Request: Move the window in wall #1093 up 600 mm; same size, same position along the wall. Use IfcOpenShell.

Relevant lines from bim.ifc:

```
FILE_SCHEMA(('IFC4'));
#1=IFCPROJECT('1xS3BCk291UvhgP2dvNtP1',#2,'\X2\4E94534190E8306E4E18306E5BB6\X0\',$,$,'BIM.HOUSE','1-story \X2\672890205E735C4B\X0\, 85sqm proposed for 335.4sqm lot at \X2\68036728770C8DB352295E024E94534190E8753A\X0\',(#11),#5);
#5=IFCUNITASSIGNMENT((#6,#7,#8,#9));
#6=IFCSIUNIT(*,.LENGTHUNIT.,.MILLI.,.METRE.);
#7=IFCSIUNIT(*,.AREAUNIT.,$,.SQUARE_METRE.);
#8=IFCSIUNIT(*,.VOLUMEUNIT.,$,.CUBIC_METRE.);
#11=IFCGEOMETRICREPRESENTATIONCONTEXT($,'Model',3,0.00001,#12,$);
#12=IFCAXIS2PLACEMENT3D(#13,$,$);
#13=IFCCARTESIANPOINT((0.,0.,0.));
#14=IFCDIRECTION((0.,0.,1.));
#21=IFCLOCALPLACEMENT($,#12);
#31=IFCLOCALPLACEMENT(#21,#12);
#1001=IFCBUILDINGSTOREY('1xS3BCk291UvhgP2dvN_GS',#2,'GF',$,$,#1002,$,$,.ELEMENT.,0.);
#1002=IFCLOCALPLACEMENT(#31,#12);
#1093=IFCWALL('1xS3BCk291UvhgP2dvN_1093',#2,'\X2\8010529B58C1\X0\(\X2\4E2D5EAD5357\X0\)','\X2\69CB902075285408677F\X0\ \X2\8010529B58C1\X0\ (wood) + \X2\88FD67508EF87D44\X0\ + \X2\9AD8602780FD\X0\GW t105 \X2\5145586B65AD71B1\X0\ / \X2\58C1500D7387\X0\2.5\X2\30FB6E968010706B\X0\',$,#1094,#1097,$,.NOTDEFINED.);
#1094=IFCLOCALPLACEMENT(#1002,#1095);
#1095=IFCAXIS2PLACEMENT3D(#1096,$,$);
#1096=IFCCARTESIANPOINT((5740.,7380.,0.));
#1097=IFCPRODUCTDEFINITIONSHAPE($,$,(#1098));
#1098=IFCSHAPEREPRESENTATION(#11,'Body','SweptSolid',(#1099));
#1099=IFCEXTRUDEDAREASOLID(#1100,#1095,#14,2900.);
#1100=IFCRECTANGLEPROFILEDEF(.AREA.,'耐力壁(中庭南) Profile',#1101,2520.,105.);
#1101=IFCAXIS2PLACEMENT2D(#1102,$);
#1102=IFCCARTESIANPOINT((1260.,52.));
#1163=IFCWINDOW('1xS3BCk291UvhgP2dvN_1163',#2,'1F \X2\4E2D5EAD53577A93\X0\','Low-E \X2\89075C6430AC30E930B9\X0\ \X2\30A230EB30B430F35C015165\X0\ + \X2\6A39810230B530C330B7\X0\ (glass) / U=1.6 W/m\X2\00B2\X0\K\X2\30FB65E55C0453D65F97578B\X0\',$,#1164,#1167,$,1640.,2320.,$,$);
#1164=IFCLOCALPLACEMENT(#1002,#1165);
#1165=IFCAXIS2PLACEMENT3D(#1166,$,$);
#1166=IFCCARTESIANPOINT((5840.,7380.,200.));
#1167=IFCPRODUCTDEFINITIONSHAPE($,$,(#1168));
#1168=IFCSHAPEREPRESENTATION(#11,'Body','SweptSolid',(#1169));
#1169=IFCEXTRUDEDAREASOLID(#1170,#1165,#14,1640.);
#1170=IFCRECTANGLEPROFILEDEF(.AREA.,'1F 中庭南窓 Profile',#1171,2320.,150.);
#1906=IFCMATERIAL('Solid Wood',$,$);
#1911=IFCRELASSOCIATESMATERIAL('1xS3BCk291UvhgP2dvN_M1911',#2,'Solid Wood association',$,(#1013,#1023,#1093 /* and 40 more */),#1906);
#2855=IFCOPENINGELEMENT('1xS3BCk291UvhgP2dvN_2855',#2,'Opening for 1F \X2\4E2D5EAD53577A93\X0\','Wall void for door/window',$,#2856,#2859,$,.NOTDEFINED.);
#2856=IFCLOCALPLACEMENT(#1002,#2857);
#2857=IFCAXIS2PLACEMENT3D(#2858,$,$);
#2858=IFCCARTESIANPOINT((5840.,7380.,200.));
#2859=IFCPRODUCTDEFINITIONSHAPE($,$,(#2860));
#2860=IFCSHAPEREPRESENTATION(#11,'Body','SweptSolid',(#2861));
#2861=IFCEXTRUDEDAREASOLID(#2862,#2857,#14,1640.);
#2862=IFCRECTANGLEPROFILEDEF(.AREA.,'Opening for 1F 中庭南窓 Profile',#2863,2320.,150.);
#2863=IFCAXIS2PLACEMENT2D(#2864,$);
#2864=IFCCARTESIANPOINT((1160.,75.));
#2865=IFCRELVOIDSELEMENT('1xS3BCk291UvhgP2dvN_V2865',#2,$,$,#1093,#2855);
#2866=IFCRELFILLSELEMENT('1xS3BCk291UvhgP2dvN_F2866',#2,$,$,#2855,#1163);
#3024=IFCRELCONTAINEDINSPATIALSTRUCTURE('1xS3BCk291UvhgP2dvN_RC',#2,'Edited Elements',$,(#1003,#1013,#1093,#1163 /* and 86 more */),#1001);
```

```python
import numpy as np
import ifcopenshell
import ifcopenshell.api.geometry
import ifcopenshell.util.placement
import ifcopenshell.util.unit

model = ifcopenshell.open("bim.ifc")
unit_scale = ifcopenshell.util.unit.calculate_unit_scale(model)

window = model.by_guid("1xS3BCk291UvhgP2dvN_1163")
opening = window.FillsVoids[0].RelatingOpeningElement
dz = 0.6 / unit_scale

shift = np.array([0.0, 0.0, dz])
# The window is not placed relative to its opening, so move both.
for product in (opening, window):
    matrix = ifcopenshell.util.placement.get_local_placement(product.ObjectPlacement)
    matrix[:3, 3] += shift
    ifcopenshell.api.geometry.edit_object_placement(model, product=product, matrix=matrix, is_si=False)

print(f"moved by {dz * unit_scale:+.3f} m")

model.write("bim-out.ifc")
```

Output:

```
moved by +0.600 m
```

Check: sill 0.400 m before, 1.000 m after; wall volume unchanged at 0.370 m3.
